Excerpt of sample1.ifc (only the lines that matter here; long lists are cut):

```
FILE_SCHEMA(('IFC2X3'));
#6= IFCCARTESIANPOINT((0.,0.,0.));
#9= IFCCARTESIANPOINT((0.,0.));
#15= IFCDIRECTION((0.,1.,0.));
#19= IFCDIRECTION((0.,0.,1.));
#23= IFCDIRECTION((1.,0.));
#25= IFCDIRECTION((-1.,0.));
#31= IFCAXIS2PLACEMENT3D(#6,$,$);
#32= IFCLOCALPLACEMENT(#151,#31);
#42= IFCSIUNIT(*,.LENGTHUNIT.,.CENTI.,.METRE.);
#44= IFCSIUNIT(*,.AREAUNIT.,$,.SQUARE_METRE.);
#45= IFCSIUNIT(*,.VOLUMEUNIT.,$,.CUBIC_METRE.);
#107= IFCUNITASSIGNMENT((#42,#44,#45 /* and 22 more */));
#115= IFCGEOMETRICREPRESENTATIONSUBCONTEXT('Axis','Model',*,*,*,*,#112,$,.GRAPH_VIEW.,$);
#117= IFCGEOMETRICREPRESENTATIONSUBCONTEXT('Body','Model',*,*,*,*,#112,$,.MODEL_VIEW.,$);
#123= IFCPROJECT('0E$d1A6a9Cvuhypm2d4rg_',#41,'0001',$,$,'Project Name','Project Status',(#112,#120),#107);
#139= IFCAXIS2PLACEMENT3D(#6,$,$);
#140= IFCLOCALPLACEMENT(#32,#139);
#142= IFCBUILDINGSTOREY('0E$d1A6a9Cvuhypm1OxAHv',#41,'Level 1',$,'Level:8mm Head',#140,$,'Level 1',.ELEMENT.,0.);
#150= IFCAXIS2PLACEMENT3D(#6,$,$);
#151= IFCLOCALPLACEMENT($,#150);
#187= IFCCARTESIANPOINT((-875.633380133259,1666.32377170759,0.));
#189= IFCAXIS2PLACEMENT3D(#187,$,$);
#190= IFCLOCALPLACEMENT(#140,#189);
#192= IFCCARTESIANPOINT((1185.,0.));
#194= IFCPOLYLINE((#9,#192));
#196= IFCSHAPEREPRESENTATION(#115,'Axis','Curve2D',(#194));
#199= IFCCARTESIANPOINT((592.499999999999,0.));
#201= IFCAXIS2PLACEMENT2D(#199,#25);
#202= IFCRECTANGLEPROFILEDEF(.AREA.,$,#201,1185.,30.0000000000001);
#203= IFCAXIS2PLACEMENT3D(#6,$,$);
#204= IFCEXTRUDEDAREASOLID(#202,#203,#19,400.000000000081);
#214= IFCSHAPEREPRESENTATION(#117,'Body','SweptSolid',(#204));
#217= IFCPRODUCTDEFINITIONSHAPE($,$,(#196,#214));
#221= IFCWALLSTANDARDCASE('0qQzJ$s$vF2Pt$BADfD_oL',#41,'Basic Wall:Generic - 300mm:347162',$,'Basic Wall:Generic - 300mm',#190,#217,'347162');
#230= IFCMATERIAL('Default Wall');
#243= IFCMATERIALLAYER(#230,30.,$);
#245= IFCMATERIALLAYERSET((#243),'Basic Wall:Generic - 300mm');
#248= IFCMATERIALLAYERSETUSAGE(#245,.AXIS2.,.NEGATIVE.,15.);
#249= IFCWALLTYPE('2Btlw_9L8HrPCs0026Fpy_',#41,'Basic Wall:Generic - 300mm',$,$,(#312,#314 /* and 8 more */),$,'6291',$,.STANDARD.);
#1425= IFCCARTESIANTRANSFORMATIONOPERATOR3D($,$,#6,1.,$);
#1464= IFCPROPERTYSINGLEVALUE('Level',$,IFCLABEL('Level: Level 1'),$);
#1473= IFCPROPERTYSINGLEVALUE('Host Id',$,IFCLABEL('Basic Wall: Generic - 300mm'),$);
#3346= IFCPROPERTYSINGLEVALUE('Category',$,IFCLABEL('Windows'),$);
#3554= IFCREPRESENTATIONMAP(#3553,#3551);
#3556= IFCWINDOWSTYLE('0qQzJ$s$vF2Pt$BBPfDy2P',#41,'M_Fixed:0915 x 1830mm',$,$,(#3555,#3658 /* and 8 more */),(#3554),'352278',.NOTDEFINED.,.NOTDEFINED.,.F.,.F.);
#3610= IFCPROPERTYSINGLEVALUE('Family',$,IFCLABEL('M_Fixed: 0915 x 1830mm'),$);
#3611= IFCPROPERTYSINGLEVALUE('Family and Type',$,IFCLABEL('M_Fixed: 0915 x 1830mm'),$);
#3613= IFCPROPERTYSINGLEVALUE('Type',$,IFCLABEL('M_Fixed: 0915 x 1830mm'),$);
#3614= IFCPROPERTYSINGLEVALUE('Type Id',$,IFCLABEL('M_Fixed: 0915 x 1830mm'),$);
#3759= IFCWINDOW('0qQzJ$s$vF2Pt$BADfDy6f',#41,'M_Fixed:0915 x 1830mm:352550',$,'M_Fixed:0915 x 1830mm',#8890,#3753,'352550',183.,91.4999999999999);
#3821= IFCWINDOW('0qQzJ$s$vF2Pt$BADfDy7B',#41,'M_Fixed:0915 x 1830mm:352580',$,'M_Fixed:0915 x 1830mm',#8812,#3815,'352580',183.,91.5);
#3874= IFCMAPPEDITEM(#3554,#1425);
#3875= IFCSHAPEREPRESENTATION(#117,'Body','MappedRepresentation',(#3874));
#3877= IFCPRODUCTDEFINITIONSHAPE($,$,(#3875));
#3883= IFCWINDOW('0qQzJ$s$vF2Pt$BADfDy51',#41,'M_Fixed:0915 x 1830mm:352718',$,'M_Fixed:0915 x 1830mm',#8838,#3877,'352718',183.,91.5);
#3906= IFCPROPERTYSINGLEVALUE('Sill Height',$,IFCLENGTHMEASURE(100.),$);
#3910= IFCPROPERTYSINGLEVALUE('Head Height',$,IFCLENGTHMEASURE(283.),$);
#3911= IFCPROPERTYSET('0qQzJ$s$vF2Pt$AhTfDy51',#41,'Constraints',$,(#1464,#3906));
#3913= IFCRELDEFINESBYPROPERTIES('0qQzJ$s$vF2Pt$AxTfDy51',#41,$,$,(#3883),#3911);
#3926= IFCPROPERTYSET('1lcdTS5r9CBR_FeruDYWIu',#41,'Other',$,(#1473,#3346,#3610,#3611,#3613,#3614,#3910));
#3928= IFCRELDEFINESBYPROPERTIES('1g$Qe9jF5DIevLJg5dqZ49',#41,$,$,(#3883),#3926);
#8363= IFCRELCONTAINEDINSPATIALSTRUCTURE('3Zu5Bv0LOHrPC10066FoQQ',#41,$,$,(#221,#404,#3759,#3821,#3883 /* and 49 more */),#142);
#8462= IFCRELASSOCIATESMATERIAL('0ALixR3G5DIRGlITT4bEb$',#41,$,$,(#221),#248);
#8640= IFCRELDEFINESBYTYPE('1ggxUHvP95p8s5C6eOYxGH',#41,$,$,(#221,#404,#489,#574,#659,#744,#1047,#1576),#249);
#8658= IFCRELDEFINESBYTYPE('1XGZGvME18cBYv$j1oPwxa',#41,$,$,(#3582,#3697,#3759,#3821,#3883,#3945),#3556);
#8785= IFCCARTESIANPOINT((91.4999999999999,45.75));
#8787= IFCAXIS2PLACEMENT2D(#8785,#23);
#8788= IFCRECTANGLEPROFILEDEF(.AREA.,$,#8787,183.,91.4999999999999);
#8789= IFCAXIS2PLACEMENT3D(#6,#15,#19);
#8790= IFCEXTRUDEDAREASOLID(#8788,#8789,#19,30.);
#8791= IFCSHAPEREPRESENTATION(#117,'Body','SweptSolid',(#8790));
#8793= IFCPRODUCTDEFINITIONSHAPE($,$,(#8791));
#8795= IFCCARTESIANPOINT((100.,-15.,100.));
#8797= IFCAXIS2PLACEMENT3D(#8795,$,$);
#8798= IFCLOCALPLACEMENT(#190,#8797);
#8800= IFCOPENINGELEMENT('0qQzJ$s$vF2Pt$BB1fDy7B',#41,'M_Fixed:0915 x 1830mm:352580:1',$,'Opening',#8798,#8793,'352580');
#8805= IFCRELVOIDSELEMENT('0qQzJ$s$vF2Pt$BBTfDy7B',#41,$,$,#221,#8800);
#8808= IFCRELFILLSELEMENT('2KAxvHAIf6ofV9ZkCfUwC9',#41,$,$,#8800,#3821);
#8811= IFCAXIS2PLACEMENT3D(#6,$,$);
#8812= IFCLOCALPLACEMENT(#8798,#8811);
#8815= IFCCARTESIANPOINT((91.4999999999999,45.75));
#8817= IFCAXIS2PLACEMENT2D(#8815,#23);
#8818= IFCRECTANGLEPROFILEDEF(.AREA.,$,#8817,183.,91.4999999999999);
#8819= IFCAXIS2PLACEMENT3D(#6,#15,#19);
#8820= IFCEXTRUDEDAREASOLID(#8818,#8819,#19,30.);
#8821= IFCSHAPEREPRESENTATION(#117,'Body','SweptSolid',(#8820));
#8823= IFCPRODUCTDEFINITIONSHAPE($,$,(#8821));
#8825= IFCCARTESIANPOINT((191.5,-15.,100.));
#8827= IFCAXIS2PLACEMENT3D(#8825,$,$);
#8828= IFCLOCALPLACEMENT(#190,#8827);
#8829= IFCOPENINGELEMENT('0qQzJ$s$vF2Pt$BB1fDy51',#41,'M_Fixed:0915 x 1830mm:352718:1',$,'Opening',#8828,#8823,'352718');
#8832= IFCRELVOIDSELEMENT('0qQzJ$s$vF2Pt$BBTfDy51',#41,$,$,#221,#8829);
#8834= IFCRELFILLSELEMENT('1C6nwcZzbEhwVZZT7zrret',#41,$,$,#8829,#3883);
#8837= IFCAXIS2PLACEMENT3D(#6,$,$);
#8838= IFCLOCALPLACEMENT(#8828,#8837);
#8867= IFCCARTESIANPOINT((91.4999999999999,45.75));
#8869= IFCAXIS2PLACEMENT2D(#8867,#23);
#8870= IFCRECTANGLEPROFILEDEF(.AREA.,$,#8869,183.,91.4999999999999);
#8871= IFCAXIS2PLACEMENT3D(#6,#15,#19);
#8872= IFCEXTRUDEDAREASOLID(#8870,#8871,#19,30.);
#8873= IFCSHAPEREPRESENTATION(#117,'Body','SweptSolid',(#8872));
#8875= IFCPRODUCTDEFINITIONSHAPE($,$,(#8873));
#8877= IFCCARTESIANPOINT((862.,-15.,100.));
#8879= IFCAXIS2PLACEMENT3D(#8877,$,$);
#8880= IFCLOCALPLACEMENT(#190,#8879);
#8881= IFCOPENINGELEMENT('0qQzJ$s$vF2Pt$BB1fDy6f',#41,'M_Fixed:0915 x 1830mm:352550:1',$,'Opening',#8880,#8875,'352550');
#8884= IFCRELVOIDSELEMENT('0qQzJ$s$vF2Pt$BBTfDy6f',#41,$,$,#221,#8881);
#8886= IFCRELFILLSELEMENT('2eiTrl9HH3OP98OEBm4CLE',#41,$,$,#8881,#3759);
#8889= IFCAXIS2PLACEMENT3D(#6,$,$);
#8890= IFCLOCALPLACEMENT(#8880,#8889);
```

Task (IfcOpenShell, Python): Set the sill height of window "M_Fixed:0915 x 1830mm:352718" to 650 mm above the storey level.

```python
import numpy as np
import ifcopenshell
import ifcopenshell.api.geometry
import ifcopenshell.api.pset
import ifcopenshell.geom
import ifcopenshell.util.element
import ifcopenshell.util.placement
import ifcopenshell.util.shape
import ifcopenshell.util.unit

model = ifcopenshell.open("sample1.ifc")
unit_scale = ifcopenshell.util.unit.calculate_unit_scale(model)

window = model.by_guid("0qQzJ$s$vF2Pt$BADfDy51")
opening = window.FillsVoids[0].RelatingOpeningElement
storey = ifcopenshell.util.element.get_container(window, ifc_class="IfcBuildingStorey")
level = ifcopenshell.util.placement.get_local_placement(storey.ObjectPlacement)[2, 3]

# The opening's origin need not be at the sill, so measure its lowest point.
shape = ifcopenshell.geom.create_shape(ifcopenshell.geom.settings(), opening)
bottom = ifcopenshell.util.shape.get_shape_bottom_elevation(shape, shape.geometry) / unit_scale
dz = level + 0.65 / unit_scale - bottom

shift = np.array([0.0, 0.0, dz])
# The window is placed relative to its opening, so it follows when the opening moves.
matrix = ifcopenshell.util.placement.get_local_placement(opening.ObjectPlacement)
matrix[:3, 3] += shift
ifcopenshell.api.geometry.edit_object_placement(
    model, product=opening, matrix=matrix, is_si=False, should_transform_children=True
)

# Keep the stored heights in step.
pset = model.by_id(ifcopenshell.util.element.get_pset(window, "Constraints", should_inherit=False)["id"])
ifcopenshell.api.pset.edit_pset(model, pset=pset, properties={
    "Sill Height": model.create_entity("IfcLengthMeasure", ifcopenshell.util.element.get_pset(window, "Constraints", "Sill Height") + dz),
})
pset = model.by_id(ifcopenshell.util.element.get_pset(window, "Other", should_inherit=False)["id"])
ifcopenshell.api.pset.edit_pset(model, pset=pset, properties={
    "Head Height": model.create_entity("IfcLengthMeasure", ifcopenshell.util.element.get_pset(window, "Other", "Head Height") + dz),
})

print(f"moved by {dz * unit_scale:+.3f} m")

model.write("sample1_updated.ifc")
```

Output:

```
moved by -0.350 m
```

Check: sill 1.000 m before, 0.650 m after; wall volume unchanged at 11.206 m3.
